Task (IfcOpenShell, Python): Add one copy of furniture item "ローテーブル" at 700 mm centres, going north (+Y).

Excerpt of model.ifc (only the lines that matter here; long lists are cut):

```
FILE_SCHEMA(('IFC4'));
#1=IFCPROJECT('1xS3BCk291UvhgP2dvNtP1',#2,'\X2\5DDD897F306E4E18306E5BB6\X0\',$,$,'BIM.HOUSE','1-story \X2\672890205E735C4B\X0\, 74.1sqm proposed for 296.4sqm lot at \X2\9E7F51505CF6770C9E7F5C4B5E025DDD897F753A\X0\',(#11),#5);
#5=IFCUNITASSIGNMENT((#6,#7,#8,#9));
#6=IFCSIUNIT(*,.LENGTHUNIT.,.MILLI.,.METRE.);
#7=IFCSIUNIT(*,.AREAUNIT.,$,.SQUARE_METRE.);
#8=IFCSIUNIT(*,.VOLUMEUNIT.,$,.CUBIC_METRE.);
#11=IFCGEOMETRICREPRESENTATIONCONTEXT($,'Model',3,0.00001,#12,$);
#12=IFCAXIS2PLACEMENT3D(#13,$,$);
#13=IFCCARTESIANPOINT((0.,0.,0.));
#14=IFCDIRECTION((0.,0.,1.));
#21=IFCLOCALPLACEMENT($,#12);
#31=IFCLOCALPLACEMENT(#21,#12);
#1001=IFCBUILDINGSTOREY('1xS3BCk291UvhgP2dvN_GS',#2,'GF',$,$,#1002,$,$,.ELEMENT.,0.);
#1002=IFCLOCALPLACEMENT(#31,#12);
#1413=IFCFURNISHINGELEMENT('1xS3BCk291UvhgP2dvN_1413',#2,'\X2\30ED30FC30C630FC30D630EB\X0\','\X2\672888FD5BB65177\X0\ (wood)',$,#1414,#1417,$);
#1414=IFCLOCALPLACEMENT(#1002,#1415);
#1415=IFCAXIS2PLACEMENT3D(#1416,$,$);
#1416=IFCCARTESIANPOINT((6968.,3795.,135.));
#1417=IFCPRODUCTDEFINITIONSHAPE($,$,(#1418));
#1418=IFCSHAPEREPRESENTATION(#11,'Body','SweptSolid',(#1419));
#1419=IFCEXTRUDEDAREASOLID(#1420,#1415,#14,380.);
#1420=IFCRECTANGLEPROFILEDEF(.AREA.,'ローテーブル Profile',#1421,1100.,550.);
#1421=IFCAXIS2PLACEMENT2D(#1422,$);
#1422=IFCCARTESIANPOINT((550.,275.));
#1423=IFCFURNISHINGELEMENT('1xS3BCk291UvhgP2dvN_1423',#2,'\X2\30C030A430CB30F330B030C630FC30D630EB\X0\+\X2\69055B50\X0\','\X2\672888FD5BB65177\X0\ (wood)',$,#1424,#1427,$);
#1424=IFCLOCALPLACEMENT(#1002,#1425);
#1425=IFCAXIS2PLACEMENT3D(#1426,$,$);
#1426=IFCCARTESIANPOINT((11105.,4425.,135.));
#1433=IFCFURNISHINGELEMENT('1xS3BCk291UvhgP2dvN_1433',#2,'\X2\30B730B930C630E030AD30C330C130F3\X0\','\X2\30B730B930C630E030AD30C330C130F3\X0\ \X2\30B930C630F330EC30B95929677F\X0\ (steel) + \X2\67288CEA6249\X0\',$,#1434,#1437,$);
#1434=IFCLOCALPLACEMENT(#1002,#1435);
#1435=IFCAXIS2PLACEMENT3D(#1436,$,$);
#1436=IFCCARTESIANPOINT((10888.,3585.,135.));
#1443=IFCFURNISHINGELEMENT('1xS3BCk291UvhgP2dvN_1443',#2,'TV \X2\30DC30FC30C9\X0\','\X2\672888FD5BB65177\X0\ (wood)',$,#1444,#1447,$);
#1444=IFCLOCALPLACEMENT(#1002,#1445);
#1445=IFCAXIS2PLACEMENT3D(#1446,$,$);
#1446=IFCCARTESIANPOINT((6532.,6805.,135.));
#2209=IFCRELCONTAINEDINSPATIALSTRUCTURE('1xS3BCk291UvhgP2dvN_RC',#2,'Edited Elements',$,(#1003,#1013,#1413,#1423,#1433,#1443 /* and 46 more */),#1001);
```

```python
import numpy as np
import ifcopenshell
import ifcopenshell.api.geometry
import ifcopenshell.api.root
import ifcopenshell.util.element
import ifcopenshell.util.placement
import ifcopenshell.util.unit

model = ifcopenshell.open("model.ifc")
unit_scale = ifcopenshell.util.unit.calculate_unit_scale(model)


def reuse_history(source, copy):
    """copy_class also copies each property set's owner history, people and application; keep the originals."""
    for rel in copy.IsDefinedBy:
        if rel.is_a("IfcRelDefinesByProperties") and (history := rel.RelatingPropertyDefinition.OwnerHistory):
            rel.RelatingPropertyDefinition.OwnerHistory = source.OwnerHistory
            ifcopenshell.util.element.remove_deep2(model, history)


source = model.by_guid("1xS3BCk291UvhgP2dvN_1413")
base = ifcopenshell.util.placement.get_local_placement(source.ObjectPlacement)
step = np.array([0.0, 1.0, 0.0]) * 0.7 / unit_scale

for i in range(1, 2):
    copy = ifcopenshell.api.root.copy_class(model, product=source)
    copy.Representation = ifcopenshell.util.element.copy_deep(
        model, source.Representation, exclude=["IfcGeometricRepresentationContext", "IfcRepresentationMap"]
    )
    reuse_history(source, copy)
    matrix = base.copy()
    matrix[:3, 3] += i * step
    print("added at", matrix[:3, 3].round(3) + 0.0)
    ifcopenshell.api.geometry.edit_object_placement(model, product=copy, matrix=matrix, is_si=False)

model.write("model_edited.ifc")
```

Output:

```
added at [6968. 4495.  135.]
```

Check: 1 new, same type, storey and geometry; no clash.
